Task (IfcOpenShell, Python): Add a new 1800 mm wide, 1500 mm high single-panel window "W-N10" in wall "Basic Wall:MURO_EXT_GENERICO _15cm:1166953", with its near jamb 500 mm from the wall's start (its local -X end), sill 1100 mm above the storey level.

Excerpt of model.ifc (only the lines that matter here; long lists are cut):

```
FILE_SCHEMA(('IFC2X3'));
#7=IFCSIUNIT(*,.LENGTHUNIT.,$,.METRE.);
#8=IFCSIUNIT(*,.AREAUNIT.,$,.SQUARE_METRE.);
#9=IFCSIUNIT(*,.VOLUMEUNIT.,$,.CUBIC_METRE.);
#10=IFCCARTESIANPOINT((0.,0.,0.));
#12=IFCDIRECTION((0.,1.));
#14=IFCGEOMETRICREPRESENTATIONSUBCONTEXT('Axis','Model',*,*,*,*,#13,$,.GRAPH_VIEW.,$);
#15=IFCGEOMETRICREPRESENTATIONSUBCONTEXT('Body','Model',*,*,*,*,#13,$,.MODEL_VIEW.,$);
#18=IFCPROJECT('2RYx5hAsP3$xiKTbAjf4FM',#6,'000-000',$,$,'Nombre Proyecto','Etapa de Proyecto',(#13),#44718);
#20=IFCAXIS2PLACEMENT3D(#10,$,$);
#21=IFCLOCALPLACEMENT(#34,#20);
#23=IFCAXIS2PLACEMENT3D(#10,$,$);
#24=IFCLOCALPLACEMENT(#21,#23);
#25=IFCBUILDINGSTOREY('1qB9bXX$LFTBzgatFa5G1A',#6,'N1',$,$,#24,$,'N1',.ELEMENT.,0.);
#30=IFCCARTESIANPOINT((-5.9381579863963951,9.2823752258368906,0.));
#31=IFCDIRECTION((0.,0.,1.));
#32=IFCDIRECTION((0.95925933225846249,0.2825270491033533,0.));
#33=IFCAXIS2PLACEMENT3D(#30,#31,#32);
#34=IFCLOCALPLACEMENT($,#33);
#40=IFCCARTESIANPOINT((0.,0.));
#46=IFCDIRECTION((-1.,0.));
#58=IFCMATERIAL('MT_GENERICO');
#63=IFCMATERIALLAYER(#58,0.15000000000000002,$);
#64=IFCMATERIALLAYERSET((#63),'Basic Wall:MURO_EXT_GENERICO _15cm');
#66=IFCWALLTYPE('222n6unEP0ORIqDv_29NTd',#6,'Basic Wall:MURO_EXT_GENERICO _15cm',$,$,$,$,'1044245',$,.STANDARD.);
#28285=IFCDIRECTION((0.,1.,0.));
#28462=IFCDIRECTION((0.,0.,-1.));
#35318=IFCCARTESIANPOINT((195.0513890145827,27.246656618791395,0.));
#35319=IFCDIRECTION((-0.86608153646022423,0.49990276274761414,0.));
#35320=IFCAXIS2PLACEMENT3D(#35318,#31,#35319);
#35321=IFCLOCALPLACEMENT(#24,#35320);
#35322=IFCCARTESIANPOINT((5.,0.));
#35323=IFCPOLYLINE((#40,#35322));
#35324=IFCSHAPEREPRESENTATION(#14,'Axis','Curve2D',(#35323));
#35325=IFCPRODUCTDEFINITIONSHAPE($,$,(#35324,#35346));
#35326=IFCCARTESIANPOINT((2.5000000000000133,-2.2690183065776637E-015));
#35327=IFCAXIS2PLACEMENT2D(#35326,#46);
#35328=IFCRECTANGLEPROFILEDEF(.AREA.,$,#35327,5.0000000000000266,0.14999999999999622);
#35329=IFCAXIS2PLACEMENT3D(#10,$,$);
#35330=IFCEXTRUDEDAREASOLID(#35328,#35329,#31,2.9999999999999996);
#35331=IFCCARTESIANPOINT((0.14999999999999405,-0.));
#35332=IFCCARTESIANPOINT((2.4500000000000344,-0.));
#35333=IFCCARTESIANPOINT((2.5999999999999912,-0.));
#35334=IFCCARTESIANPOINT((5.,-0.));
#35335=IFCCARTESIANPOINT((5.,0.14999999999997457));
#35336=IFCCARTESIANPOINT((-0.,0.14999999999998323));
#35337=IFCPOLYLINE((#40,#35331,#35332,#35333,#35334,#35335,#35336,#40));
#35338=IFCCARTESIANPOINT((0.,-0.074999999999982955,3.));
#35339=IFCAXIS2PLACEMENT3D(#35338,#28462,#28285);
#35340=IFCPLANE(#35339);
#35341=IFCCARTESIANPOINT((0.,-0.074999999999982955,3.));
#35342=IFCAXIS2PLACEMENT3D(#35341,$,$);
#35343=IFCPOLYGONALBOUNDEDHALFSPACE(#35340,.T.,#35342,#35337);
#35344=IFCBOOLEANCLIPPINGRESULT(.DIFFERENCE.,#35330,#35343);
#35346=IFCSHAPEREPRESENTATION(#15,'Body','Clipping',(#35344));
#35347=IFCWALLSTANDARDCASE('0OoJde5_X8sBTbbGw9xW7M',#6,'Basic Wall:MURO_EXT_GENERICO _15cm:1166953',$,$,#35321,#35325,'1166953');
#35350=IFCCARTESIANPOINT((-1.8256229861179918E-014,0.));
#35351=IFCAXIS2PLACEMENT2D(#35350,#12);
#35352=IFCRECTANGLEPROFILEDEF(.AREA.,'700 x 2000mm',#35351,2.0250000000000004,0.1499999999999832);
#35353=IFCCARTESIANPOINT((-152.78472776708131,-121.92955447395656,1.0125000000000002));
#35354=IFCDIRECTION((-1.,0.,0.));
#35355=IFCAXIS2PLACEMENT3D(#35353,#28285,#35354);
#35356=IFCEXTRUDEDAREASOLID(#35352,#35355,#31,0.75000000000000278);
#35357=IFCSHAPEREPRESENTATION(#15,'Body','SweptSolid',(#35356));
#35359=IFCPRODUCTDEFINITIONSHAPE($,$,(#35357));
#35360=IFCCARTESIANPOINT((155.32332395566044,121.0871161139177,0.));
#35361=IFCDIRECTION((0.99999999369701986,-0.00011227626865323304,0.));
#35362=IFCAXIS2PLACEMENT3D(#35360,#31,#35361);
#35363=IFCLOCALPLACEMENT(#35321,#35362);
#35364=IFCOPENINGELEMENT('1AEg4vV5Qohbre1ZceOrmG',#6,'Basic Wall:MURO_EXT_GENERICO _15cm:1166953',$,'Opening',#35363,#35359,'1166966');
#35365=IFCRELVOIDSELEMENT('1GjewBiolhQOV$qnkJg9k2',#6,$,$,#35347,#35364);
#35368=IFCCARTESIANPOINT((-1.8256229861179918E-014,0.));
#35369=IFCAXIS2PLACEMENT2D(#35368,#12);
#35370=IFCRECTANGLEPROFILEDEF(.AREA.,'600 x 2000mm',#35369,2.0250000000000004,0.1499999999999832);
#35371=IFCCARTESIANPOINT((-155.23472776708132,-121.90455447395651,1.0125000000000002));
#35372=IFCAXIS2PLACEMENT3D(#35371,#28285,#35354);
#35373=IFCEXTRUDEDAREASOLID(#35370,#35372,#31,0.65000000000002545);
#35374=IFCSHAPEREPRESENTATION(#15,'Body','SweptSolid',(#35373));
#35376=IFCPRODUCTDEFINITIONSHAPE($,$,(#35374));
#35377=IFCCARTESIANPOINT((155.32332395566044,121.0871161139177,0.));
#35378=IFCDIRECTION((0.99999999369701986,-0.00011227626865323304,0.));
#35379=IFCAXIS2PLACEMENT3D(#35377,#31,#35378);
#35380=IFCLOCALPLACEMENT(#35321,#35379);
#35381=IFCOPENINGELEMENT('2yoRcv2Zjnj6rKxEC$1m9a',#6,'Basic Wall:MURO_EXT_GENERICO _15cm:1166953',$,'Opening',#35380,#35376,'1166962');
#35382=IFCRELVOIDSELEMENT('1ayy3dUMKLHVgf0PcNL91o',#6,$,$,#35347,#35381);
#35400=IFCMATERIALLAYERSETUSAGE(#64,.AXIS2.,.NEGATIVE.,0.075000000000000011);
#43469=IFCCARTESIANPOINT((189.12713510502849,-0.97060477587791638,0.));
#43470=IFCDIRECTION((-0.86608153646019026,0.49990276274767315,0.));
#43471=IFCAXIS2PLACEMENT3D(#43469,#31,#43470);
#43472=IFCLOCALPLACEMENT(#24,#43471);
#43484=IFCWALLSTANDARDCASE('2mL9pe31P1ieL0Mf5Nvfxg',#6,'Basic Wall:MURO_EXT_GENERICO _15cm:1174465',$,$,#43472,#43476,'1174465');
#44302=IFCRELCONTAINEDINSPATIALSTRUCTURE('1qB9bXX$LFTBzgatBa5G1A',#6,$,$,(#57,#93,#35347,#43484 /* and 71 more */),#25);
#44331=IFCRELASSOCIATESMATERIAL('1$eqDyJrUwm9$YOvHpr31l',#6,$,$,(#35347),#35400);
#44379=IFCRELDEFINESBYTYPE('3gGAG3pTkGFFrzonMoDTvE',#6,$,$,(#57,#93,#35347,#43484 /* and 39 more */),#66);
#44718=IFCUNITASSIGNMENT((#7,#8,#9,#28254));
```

```python
import numpy as np
import ifcopenshell
import ifcopenshell.api.feature
import ifcopenshell.api.geometry
import ifcopenshell.api.root
import ifcopenshell.api.spatial
import ifcopenshell.api.type
import ifcopenshell.geom
import ifcopenshell.util.element
import ifcopenshell.util.placement
import ifcopenshell.util.representation
import ifcopenshell.util.shape
import ifcopenshell.util.unit

model = ifcopenshell.open("model.ifc")
unit_scale = ifcopenshell.util.unit.calculate_unit_scale(model)
settings = ifcopenshell.geom.settings()


def volume(element):
    """Net volume in cubic metres, openings subtracted."""
    shape = ifcopenshell.geom.create_shape(settings, element)
    return ifcopenshell.util.shape.get_volume(shape.geometry)


wall = model.by_guid("0OoJde5_X8sBTbbGw9xW7M")
storey = ifcopenshell.util.element.get_container(wall, ifc_class="IfcBuildingStorey")
context = ifcopenshell.util.representation.get_context(model, "Model", "Body", "MODEL_VIEW")
before = volume(wall)

width, height, from_end, sill = 1.8, 1.5, 0.5, 1.1  # metres

# The wall runs along its own X axis, and the end named is its -X end.
wall_shape = ifcopenshell.geom.create_shape(settings, wall)
x, y, z = ifcopenshell.util.shape.get_vertices(wall_shape.geometry).T
start = x.min() + from_end
face, thickness = float(y.min()), float(y.max() - y.min())
wall_matrix = ifcopenshell.util.placement.get_local_placement(wall.ObjectPlacement)
level = ifcopenshell.util.placement.get_local_placement(storey.ObjectPlacement)[2, 3]


def in_wall(x, y):
    """Placement at x, y metres in the wall's axes, at sill height."""
    matrix = wall_matrix.copy()
    matrix[:, 3] = wall_matrix @ np.array([x / unit_scale, y / unit_scale, 0.0, 1.0])
    matrix[2, 3] = level + sill / unit_scale
    return matrix


# Opening: a box that overshoots both wall faces by 50 mm.
opening = ifcopenshell.api.root.create_entity(model, ifc_class="IfcOpeningElement")
box = ifcopenshell.api.geometry.add_wall_representation(
    model, context=context, length=width, height=height, thickness=thickness + 0.1
)
ifcopenshell.api.geometry.assign_representation(model, product=opening, representation=box)
ifcopenshell.api.geometry.edit_object_placement(model, product=opening, matrix=in_wall(start, face - 0.05), is_si=False)
ifcopenshell.api.feature.add_feature(model, feature=opening, element=wall)

window = ifcopenshell.api.root.create_entity(model, ifc_class="IfcWindow", name="W-N10")
window.OverallWidth, window.OverallHeight = width / unit_scale, height / unit_scale
body = ifcopenshell.api.geometry.add_window_representation(
    model,
    context=context,
    overall_width=window.OverallWidth,
    overall_height=window.OverallHeight,
    partition_type="SINGLE_PANEL",
)
ifcopenshell.api.geometry.assign_representation(model, product=window, representation=body)
ifcopenshell.api.spatial.assign_container(model, products=[window], relating_structure=storey)
fills = ifcopenshell.api.feature.add_filling(model, opening=opening, element=window)
fills.OwnerHistory = window.OwnerHistory  # required in IFC2X3

# IFC2X3 keeps the operation on the window style.
style = ifcopenshell.api.root.create_entity(model, ifc_class="IfcWindowStyle", name="W-N10")
style.OperationType, style.ConstructionType = "SINGLE_PANEL", "NOTDEFINED"
style.ParameterTakesPrecedence = style.Sizeable = False
ifcopenshell.api.type.assign_type(model, related_objects=[window], relating_type=style)

# Centre the window in the wall's thickness.
ifcopenshell.api.geometry.edit_object_placement(model, product=window, matrix=in_wall(start, face), is_si=False)
window_shape = ifcopenshell.geom.create_shape(settings, window)
depth = ifcopenshell.util.shape.get_vertices(window_shape.geometry)[:, 1]
offset = face + thickness / 2 - (depth.min() + depth.max()) / 2
ifcopenshell.api.geometry.edit_object_placement(model, product=window, matrix=in_wall(start, offset), is_si=False)

after = volume(wall)

print(f"wall volume {before:.3f} -> {after:.3f} m3")

model.write("model-out.ifc")
```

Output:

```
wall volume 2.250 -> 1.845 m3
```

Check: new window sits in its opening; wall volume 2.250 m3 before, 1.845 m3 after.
